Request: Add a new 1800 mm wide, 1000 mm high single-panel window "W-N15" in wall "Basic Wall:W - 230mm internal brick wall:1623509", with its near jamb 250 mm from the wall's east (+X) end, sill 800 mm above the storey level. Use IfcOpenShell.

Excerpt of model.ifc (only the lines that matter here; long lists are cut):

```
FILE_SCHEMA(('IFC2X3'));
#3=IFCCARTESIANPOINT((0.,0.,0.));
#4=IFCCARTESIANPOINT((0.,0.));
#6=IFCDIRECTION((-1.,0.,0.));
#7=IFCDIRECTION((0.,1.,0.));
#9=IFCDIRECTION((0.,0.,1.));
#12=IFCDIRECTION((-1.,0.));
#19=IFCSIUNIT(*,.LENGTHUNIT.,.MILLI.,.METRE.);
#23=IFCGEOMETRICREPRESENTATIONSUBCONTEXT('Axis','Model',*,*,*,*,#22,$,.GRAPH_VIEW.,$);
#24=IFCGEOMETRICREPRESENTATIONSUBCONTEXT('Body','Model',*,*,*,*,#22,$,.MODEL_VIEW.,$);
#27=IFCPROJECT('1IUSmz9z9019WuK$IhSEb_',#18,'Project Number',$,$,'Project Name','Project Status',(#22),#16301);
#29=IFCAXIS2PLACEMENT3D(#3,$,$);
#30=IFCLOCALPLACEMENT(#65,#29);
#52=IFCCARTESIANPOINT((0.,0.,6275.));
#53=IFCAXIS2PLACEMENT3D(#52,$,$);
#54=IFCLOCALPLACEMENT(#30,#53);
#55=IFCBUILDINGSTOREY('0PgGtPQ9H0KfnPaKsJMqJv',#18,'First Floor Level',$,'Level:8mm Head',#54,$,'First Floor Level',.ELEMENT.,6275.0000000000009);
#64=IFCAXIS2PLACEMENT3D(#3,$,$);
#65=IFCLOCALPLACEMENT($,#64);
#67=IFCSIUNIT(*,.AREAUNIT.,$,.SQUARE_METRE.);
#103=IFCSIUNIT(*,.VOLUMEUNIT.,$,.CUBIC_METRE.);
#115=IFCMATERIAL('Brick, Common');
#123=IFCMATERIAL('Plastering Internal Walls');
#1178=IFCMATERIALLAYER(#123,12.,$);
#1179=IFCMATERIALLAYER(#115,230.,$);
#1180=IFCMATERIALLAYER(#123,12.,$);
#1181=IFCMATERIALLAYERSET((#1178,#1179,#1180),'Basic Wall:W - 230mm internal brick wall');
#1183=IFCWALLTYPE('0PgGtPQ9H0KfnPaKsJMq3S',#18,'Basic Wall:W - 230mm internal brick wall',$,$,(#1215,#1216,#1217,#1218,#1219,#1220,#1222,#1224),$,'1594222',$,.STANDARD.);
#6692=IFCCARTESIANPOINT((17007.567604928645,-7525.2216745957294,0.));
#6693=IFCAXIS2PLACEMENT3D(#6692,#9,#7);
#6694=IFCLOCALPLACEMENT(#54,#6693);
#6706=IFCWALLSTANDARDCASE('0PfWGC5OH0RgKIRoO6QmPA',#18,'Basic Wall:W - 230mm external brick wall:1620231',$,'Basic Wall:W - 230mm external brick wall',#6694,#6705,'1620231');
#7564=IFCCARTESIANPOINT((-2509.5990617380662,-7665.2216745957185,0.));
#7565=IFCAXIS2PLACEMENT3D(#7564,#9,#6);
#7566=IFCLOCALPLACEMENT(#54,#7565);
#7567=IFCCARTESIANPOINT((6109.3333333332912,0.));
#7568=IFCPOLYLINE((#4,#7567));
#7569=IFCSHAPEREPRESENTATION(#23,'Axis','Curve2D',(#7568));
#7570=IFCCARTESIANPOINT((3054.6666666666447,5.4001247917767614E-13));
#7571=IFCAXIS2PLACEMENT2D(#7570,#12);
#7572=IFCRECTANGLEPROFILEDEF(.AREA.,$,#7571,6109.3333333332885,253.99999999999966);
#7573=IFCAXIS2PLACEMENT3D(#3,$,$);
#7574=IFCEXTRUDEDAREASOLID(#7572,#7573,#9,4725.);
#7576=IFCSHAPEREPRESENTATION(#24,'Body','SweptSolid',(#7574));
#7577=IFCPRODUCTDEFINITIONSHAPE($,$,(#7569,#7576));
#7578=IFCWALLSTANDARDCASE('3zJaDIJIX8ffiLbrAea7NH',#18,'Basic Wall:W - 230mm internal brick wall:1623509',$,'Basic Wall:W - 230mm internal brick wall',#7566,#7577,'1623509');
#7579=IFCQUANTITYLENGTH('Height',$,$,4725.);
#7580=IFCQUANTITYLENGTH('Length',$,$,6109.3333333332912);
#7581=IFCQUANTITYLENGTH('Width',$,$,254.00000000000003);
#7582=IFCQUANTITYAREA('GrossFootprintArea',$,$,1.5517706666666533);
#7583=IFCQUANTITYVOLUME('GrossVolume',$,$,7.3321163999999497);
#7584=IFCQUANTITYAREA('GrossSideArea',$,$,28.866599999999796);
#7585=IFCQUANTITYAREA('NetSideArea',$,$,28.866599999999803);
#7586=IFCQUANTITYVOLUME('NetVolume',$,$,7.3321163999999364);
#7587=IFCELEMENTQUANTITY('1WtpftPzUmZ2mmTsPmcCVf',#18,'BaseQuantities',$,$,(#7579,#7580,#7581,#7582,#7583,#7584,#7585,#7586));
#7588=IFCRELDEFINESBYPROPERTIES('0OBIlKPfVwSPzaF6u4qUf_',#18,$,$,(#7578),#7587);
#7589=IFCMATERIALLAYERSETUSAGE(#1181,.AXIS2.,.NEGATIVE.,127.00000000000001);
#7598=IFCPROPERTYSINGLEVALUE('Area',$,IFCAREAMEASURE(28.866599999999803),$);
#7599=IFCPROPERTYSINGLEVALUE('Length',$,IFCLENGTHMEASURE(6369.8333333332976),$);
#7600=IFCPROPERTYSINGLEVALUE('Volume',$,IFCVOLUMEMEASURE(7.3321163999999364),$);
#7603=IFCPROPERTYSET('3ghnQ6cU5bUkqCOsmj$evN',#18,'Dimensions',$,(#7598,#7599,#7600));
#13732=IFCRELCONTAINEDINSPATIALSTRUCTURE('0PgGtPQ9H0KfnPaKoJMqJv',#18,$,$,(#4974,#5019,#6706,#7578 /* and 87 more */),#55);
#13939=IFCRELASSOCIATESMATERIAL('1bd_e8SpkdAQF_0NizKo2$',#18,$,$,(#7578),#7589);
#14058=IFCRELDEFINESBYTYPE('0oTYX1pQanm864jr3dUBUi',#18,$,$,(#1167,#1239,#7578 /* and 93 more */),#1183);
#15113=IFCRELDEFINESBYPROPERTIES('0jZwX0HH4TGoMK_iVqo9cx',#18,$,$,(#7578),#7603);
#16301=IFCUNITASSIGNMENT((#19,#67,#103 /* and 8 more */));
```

```python
import numpy as np
import ifcopenshell
import ifcopenshell.api.feature
import ifcopenshell.api.geometry
import ifcopenshell.api.pset
import ifcopenshell.api.root
import ifcopenshell.api.spatial
import ifcopenshell.api.type
import ifcopenshell.geom
import ifcopenshell.util.element
import ifcopenshell.util.placement
import ifcopenshell.util.representation
import ifcopenshell.util.shape
import ifcopenshell.util.unit

model = ifcopenshell.open("model.ifc")
unit_scale = ifcopenshell.util.unit.calculate_unit_scale(model)
area_scale = ifcopenshell.util.unit.calculate_unit_scale(model, "AREAUNIT")
volume_scale = ifcopenshell.util.unit.calculate_unit_scale(model, "VOLUMEUNIT")
settings = ifcopenshell.geom.settings()


def volume(element):
    """Net volume in cubic metres, openings subtracted."""
    shape = ifcopenshell.geom.create_shape(settings, element)
    return ifcopenshell.util.shape.get_volume(shape.geometry)


wall = model.by_guid("3zJaDIJIX8ffiLbrAea7NH")
storey = ifcopenshell.util.element.get_container(wall, ifc_class="IfcBuildingStorey")
context = ifcopenshell.util.representation.get_context(model, "Model", "Body", "MODEL_VIEW")
before = volume(wall)

width, height, from_end, sill = 1.8, 1, 0.25, 0.8  # metres

# The wall runs along its own X axis, and the end named is its -X end.
wall_shape = ifcopenshell.geom.create_shape(settings, wall)
x, y, z = ifcopenshell.util.shape.get_vertices(wall_shape.geometry).T
start = x.min() + from_end
face, thickness = float(y.min()), float(y.max() - y.min())
wall_matrix = ifcopenshell.util.placement.get_local_placement(wall.ObjectPlacement)
level = ifcopenshell.util.placement.get_local_placement(storey.ObjectPlacement)[2, 3]


def in_wall(x, y):
    """Placement at x, y metres in the wall's axes, at sill height."""
    matrix = wall_matrix.copy()
    matrix[:, 3] = wall_matrix @ np.array([x / unit_scale, y / unit_scale, 0.0, 1.0])
    matrix[2, 3] = level + sill / unit_scale
    return matrix


# Opening: a box that overshoots both wall faces by 50 mm.
opening = ifcopenshell.api.root.create_entity(model, ifc_class="IfcOpeningElement")
box = ifcopenshell.api.geometry.add_wall_representation(
    model, context=context, length=width, height=height, thickness=thickness + 0.1
)
ifcopenshell.api.geometry.assign_representation(model, product=opening, representation=box)
ifcopenshell.api.geometry.edit_object_placement(model, product=opening, matrix=in_wall(start, face - 0.05), is_si=False)
ifcopenshell.api.feature.add_feature(model, feature=opening, element=wall)

window = ifcopenshell.api.root.create_entity(model, ifc_class="IfcWindow", name="W-N15")
window.OverallWidth, window.OverallHeight = width / unit_scale, height / unit_scale
body = ifcopenshell.api.geometry.add_window_representation(
    model,
    context=context,
    overall_width=window.OverallWidth,
    overall_height=window.OverallHeight,
    partition_type="SINGLE_PANEL",
)
ifcopenshell.api.geometry.assign_representation(model, product=window, representation=body)
ifcopenshell.api.spatial.assign_container(model, products=[window], relating_structure=storey)
fills = ifcopenshell.api.feature.add_filling(model, opening=opening, element=window)
fills.OwnerHistory = window.OwnerHistory  # required in IFC2X3

# IFC2X3 keeps the operation on the window style.
style = ifcopenshell.api.root.create_entity(model, ifc_class="IfcWindowStyle", name="W-N15")
style.OperationType, style.ConstructionType = "SINGLE_PANEL", "NOTDEFINED"
style.ParameterTakesPrecedence = style.Sizeable = False
ifcopenshell.api.type.assign_type(model, related_objects=[window], relating_type=style)

# Centre the window in the wall's thickness.
ifcopenshell.api.geometry.edit_object_placement(model, product=window, matrix=in_wall(start, face), is_si=False)
window_shape = ifcopenshell.geom.create_shape(settings, window)
depth = ifcopenshell.util.shape.get_vertices(window_shape.geometry)[:, 1]
offset = face + thickness / 2 - (depth.min() + depth.max()) / 2
ifcopenshell.api.geometry.edit_object_placement(model, product=window, matrix=in_wall(start, offset), is_si=False)

after = volume(wall)

# Update the wall's stored quantities.
qto = model.by_id(ifcopenshell.util.element.get_pset(wall, "BaseQuantities", should_inherit=False)["id"])
ifcopenshell.api.pset.edit_qto(model, qto=qto, properties={
    "NetSideArea": after / thickness / area_scale,
    "NetVolume": after / volume_scale,
})
pset = model.by_id(ifcopenshell.util.element.get_pset(wall, "Dimensions", should_inherit=False)["id"])
ifcopenshell.api.pset.edit_pset(model, pset=pset, properties={
    "Area": model.create_entity("IfcAreaMeasure", after / thickness / area_scale),
    "Volume": model.create_entity("IfcVolumeMeasure", after / volume_scale),
})

print(f"wall volume {before:.3f} -> {after:.3f} m3")

model.write("model_v2.ifc")
```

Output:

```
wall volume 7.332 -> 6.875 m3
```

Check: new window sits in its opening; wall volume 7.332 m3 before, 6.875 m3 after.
